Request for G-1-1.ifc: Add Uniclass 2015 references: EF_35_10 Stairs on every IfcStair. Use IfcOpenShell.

First a look at what the model holds.

```python
import ifcopenshell

model = ifcopenshell.open("G-1-1.ifc")
print(model.schema)
print("classifications:", [c.Name for c in model.by_type("IfcClassification")])
for ifc_class in ("IfcDoor", "IfcRoof", "IfcStair", "IfcWall", "IfcWindow"):
    print(ifc_class, len(model.by_type(ifc_class)))
```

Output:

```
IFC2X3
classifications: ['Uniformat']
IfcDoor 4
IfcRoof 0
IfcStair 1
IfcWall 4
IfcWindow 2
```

```python
import ifcopenshell
import ifcopenshell.api.classification

model = ifcopenshell.open("G-1-1.ifc")

# IFC2X3 requires Source and Edition and has no link from the project to the system.
system = model.create_entity("IfcClassification", Source="NBS", Edition="2015", Name="Uniclass 2015")

codes = {
    "IfcStair": ("EF_35_10", "Stairs"),
}
for ifc_class, (code, name) in codes.items():
    products = model.by_type(ifc_class)
    ifcopenshell.api.classification.add_reference(
        model, products=products, classification=system, identification=code, name=name
    )
    print(code, len(products))

model.write("G-1-1_v2.ifc")
```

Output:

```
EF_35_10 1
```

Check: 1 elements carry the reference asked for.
